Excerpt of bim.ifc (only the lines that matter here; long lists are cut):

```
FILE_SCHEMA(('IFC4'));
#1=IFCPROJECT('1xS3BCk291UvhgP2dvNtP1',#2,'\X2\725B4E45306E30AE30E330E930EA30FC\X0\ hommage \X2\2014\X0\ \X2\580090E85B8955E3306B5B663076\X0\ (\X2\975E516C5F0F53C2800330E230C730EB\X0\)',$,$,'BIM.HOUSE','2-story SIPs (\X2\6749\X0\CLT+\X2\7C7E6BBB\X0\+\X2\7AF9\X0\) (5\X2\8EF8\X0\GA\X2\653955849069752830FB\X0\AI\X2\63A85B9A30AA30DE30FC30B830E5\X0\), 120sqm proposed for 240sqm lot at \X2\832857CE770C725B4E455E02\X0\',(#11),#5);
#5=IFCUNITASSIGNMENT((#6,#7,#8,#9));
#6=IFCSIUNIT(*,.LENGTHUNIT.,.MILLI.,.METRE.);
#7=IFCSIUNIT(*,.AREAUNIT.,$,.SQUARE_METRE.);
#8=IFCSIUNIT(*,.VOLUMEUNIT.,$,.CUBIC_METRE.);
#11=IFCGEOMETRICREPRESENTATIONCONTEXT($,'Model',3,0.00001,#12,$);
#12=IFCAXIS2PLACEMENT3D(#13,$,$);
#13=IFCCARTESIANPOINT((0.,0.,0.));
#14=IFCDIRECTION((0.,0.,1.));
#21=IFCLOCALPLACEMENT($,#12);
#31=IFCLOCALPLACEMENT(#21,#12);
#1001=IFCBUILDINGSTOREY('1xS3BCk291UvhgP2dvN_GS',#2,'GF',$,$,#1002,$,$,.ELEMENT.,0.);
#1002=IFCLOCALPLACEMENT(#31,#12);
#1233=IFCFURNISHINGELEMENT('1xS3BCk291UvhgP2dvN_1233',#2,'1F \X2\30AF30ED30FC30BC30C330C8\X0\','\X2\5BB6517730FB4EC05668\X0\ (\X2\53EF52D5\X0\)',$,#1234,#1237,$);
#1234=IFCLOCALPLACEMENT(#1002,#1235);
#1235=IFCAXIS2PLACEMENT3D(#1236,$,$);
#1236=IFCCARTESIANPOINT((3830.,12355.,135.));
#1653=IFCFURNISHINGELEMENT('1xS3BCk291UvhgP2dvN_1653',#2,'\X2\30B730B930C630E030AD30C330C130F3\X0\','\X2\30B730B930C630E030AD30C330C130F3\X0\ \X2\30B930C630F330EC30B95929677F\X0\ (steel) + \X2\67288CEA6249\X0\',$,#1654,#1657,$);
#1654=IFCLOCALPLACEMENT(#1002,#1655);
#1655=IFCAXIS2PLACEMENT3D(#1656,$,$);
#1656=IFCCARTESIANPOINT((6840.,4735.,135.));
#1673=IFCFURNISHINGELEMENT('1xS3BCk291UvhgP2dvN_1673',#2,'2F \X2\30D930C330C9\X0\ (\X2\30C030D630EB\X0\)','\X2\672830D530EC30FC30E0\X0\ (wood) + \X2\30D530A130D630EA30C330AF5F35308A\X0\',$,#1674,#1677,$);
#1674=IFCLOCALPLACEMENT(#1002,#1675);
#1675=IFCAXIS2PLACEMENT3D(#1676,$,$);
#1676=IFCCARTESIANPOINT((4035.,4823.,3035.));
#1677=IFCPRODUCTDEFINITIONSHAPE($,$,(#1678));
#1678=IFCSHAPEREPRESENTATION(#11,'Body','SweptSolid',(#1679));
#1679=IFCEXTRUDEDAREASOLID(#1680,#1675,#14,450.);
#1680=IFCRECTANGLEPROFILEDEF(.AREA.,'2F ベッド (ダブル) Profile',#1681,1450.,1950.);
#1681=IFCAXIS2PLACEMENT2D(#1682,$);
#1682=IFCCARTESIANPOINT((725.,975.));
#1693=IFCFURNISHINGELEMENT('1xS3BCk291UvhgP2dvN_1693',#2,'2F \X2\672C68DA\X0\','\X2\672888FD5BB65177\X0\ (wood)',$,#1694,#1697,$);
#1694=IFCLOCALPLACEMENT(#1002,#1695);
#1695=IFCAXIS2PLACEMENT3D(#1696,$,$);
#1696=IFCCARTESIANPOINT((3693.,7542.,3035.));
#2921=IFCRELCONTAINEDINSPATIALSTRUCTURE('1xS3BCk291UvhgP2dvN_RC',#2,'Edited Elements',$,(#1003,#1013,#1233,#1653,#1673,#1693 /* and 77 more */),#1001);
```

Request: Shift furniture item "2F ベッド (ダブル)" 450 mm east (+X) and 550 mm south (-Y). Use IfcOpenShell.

```python
import ifcopenshell
import ifcopenshell.api.geometry
import ifcopenshell.util.placement
import ifcopenshell.util.unit

model = ifcopenshell.open("bim.ifc")
unit_scale = ifcopenshell.util.unit.calculate_unit_scale(model)

item = model.by_id(1673)
matrix = ifcopenshell.util.placement.get_local_placement(item.ObjectPlacement)
matrix[0, 3] += 0.45 / unit_scale
matrix[1, 3] -= 0.55 / unit_scale
ifcopenshell.api.geometry.edit_object_placement(model, product=item, matrix=matrix, is_si=False)

print(ifcopenshell.util.placement.get_local_placement(item.ObjectPlacement).round(3) + 0.0)

model.write("bim_edited.ifc")
```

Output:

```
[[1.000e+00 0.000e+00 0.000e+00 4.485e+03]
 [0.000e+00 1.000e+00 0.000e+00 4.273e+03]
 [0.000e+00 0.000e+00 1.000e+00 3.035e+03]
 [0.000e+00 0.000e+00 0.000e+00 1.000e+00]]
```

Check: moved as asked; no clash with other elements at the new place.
